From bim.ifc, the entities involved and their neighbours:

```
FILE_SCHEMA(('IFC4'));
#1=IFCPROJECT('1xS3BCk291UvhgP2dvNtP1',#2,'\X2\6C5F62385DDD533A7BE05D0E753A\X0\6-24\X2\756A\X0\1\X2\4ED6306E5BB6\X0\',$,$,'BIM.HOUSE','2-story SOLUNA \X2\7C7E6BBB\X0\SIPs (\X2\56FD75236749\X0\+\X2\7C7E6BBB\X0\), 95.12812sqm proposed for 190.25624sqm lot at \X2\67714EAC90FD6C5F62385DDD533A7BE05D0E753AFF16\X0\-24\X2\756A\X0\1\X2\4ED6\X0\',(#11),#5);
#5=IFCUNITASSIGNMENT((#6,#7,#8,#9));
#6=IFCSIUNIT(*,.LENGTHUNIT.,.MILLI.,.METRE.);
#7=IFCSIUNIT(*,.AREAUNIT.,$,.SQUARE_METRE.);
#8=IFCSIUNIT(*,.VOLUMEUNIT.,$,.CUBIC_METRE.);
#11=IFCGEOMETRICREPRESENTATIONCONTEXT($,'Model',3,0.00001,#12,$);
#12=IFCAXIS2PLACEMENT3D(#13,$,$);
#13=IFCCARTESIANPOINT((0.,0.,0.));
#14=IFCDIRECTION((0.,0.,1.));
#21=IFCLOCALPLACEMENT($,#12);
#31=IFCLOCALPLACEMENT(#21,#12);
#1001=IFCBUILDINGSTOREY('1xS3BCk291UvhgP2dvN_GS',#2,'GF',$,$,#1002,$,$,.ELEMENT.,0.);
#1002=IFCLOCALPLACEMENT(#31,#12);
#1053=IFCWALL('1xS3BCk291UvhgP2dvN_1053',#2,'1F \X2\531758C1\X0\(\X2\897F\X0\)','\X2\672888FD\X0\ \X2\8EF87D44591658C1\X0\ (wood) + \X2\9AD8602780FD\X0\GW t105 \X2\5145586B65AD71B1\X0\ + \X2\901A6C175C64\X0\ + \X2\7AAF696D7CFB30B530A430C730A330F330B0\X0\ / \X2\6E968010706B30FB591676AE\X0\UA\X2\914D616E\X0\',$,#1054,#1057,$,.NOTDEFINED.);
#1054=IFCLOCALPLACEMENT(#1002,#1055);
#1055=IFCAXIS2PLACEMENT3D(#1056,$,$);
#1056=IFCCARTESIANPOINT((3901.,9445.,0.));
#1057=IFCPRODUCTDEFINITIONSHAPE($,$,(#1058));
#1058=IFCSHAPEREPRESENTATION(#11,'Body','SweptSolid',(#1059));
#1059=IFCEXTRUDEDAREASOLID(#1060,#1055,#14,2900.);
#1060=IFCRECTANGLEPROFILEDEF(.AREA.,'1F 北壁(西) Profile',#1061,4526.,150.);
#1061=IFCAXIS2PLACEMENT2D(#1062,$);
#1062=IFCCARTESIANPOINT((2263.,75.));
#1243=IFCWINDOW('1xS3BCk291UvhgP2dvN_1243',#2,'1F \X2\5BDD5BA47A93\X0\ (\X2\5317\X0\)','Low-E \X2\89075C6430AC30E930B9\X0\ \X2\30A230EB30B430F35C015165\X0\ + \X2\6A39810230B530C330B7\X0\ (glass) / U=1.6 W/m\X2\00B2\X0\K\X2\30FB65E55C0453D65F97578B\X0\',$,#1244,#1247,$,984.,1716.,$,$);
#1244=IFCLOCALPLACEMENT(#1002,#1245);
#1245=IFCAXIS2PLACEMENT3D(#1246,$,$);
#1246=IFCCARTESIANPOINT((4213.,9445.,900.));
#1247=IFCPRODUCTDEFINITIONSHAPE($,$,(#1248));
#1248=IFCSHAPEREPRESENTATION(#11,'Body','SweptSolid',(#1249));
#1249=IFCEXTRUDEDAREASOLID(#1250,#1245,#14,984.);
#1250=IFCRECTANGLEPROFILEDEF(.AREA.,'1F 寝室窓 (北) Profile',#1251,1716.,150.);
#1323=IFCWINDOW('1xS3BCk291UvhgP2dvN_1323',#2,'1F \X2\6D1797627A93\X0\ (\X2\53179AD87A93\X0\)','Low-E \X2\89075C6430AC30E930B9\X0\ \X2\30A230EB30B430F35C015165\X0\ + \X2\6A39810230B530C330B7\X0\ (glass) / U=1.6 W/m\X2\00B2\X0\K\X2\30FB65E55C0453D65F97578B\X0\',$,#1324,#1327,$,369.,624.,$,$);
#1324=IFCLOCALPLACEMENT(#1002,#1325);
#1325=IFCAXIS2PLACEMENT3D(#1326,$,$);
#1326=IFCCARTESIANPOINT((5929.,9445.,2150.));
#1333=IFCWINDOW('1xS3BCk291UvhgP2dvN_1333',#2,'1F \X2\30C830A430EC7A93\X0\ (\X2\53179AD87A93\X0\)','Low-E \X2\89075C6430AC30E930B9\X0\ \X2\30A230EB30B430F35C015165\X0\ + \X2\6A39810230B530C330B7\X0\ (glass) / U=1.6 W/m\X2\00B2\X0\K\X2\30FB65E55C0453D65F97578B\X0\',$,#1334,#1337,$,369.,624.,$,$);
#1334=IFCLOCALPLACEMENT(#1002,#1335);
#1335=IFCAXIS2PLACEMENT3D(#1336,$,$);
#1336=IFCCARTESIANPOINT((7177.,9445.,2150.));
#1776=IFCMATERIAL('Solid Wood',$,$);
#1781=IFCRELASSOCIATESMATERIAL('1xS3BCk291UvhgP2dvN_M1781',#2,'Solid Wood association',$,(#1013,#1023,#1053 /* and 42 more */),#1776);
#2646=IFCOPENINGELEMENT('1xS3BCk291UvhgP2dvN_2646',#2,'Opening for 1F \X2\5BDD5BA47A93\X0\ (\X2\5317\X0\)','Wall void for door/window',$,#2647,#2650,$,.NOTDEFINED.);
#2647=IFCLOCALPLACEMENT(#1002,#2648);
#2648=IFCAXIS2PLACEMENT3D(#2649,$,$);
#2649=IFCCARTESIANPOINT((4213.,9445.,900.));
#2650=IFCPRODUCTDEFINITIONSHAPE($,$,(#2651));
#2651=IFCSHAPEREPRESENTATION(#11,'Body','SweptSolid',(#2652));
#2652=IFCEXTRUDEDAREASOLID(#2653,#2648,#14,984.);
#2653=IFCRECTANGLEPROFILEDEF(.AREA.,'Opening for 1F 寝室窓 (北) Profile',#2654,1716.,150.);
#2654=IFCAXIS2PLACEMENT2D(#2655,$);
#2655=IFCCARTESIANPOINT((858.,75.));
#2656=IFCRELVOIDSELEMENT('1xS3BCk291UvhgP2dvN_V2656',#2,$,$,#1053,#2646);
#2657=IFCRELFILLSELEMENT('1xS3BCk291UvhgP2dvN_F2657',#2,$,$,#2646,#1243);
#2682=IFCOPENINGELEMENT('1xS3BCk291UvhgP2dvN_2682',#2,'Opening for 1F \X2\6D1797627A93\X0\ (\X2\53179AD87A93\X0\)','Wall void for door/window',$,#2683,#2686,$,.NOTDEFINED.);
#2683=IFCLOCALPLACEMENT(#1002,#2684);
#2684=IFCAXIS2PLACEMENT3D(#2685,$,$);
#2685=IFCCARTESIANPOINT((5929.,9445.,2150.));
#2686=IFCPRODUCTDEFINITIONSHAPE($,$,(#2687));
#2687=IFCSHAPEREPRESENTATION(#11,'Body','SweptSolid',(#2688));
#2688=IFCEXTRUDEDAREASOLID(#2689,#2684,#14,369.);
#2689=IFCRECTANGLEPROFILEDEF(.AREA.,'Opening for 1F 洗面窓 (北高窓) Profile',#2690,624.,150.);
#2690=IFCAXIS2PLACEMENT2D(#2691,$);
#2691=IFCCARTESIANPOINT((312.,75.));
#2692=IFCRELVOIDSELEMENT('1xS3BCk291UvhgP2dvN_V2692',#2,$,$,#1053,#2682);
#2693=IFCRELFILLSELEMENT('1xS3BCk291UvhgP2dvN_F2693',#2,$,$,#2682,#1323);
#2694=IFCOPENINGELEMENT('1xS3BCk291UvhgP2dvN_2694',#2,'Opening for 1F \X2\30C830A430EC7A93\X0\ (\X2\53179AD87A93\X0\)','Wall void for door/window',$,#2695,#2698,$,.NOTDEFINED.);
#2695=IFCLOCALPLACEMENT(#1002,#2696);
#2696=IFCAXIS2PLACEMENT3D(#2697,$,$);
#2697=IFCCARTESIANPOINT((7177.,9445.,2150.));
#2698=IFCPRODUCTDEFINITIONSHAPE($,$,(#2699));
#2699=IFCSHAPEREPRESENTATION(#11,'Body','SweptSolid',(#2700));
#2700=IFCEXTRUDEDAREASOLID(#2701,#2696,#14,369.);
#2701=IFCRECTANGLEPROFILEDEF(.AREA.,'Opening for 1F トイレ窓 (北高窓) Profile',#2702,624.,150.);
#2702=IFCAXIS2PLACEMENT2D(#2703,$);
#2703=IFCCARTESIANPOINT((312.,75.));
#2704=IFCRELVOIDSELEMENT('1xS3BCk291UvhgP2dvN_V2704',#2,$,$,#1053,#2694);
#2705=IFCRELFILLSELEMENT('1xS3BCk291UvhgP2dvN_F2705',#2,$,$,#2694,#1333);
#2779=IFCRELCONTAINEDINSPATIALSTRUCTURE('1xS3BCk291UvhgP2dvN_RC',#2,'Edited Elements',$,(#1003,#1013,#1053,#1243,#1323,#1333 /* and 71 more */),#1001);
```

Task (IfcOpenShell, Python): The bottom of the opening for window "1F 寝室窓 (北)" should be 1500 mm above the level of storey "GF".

```python
import numpy as np
import ifcopenshell
import ifcopenshell.api.geometry
import ifcopenshell.geom
import ifcopenshell.util.element
import ifcopenshell.util.placement
import ifcopenshell.util.shape
import ifcopenshell.util.unit

model = ifcopenshell.open("bim.ifc")
unit_scale = ifcopenshell.util.unit.calculate_unit_scale(model)

window = model.by_guid("1xS3BCk291UvhgP2dvN_1243")
opening = window.FillsVoids[0].RelatingOpeningElement
storey = ifcopenshell.util.element.get_container(window, ifc_class="IfcBuildingStorey")
level = ifcopenshell.util.placement.get_local_placement(storey.ObjectPlacement)[2, 3]

# The opening's origin need not be at the sill, so measure its lowest point.
shape = ifcopenshell.geom.create_shape(ifcopenshell.geom.settings(), opening)
bottom = ifcopenshell.util.shape.get_shape_bottom_elevation(shape, shape.geometry) / unit_scale
dz = level + 1500.0 - bottom

shift = np.array([0.0, 0.0, dz])
# The window is not placed relative to its opening, so move both.
for product in (opening, window):
    matrix = ifcopenshell.util.placement.get_local_placement(product.ObjectPlacement)
    matrix[:3, 3] += shift
    ifcopenshell.api.geometry.edit_object_placement(model, product=product, matrix=matrix, is_si=False)

print(f"moved by {dz * unit_scale:+.3f} m")

model.write("bim_v2.ifc")
```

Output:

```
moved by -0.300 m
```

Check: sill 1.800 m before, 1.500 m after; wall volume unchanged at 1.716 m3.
